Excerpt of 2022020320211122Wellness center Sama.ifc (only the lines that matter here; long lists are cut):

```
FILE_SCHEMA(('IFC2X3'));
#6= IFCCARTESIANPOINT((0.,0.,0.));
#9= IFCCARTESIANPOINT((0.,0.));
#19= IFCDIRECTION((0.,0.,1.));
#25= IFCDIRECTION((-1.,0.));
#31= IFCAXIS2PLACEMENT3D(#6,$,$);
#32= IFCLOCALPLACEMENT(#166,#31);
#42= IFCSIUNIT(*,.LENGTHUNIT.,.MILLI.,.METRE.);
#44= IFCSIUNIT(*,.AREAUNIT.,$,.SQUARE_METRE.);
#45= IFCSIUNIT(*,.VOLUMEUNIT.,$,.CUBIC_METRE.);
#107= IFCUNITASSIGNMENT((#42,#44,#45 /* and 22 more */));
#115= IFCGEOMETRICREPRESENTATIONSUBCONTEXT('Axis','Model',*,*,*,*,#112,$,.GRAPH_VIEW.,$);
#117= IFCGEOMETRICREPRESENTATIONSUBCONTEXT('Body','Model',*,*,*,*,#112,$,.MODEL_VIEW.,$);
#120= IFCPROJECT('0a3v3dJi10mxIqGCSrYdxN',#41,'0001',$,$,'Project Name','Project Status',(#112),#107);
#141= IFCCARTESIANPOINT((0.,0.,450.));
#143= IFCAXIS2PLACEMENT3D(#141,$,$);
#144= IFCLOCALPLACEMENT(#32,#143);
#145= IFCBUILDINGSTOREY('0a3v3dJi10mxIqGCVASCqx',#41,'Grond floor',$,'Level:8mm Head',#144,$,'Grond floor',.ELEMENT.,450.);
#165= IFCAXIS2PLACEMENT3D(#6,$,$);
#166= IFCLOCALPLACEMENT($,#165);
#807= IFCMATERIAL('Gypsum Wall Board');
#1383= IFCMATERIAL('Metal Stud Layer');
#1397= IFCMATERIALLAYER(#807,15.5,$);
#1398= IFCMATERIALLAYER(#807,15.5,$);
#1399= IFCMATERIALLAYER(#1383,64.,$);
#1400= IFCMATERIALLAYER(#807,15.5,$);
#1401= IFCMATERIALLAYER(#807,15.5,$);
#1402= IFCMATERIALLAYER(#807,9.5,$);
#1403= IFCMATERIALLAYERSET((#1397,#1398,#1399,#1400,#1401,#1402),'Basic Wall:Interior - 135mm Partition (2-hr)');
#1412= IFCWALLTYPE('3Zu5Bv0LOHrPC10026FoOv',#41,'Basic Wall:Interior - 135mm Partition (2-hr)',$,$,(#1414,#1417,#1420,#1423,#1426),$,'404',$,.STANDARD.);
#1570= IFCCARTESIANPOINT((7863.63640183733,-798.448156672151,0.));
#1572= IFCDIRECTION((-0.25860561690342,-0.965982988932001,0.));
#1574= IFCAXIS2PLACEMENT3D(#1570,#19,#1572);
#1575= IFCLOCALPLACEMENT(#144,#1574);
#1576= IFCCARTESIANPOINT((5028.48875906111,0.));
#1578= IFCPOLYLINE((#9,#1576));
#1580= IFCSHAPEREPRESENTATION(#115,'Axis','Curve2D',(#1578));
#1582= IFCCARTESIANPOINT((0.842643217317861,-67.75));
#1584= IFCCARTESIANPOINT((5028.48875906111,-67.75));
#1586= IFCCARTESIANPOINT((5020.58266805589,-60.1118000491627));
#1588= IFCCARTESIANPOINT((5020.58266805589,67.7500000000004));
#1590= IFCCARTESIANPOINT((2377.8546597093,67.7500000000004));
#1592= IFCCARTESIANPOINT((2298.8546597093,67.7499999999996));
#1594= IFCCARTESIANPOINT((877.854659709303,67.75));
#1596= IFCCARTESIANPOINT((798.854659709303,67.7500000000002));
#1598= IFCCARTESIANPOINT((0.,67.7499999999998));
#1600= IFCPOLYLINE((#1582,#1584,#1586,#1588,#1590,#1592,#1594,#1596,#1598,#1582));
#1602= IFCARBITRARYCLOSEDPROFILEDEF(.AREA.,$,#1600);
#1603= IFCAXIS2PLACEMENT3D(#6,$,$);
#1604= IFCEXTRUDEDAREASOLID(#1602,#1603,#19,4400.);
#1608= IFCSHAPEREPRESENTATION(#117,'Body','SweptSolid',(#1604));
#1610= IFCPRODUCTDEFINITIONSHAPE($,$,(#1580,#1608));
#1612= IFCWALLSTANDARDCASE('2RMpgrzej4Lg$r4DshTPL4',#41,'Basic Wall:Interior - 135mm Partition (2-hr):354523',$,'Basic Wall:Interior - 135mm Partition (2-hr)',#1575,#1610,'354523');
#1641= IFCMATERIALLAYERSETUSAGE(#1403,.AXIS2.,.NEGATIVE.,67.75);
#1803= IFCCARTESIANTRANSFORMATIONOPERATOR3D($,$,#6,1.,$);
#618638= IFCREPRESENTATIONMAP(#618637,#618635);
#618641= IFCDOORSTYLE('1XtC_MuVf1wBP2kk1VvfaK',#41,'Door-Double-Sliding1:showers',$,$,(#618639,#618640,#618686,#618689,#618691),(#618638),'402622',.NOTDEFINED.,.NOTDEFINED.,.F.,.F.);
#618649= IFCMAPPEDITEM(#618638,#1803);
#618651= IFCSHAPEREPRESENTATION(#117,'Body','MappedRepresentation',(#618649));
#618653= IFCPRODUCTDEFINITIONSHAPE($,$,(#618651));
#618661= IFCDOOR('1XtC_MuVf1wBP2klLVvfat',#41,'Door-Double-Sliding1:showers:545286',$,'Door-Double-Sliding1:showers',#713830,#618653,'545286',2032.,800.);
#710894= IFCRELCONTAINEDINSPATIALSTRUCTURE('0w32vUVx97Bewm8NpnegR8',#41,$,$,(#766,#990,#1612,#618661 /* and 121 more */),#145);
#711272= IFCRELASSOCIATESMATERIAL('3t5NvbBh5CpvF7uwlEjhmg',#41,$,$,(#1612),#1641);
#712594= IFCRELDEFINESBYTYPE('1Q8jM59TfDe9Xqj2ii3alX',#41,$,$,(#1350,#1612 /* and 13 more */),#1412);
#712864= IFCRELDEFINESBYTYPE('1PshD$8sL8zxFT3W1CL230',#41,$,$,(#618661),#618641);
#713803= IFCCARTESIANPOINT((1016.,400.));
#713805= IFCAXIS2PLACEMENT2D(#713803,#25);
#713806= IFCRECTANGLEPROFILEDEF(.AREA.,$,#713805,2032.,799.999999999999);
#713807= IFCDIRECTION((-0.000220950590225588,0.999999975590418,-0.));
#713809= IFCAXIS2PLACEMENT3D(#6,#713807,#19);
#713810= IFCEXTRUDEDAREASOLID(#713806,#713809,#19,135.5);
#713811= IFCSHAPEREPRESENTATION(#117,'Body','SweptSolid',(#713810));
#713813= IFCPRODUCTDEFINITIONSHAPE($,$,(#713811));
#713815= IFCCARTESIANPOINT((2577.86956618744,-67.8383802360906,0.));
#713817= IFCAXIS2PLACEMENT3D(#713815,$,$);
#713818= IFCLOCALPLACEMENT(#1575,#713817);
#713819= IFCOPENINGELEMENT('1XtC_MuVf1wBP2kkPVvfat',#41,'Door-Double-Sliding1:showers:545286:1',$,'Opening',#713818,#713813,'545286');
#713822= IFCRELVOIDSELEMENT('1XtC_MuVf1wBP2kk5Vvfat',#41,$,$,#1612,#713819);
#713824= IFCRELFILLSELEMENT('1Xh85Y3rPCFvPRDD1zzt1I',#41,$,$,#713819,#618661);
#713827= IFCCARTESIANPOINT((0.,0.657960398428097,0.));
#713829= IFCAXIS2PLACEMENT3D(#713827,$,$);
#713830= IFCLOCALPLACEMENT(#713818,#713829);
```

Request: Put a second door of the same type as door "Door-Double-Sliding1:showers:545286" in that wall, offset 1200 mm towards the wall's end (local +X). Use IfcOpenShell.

```python
import ifcopenshell
import ifcopenshell.api.feature
import ifcopenshell.api.geometry
import ifcopenshell.api.root
import ifcopenshell.geom
import ifcopenshell.util.element
import ifcopenshell.util.placement
import ifcopenshell.util.shape
import ifcopenshell.util.unit

model = ifcopenshell.open("2022020320211122Wellness center Sama.ifc")
unit_scale = ifcopenshell.util.unit.calculate_unit_scale(model)
settings = ifcopenshell.geom.settings()


def volume(element):
    """Net volume in cubic metres, openings subtracted."""
    shape = ifcopenshell.geom.create_shape(settings, element)
    return ifcopenshell.util.shape.get_volume(shape.geometry)


def reuse_history(source, copy):
    """copy_class also copies each property set's owner history, people and application; keep the originals."""
    for rel in copy.IsDefinedBy:
        if rel.is_a("IfcRelDefinesByProperties") and (history := rel.RelatingPropertyDefinition.OwnerHistory):
            rel.RelatingPropertyDefinition.OwnerHistory = source.OwnerHistory
            ifcopenshell.util.element.remove_deep2(model, history)


door = model.by_id(618661)
opening = door.FillsVoids[0].RelatingOpeningElement
wall = opening.VoidsElements[0].RelatingBuildingElement
before = volume(wall)
shift = ifcopenshell.util.placement.get_local_placement(wall.ObjectPlacement)[:3, 0] * 1.2 / unit_scale

# copy_class copies the void relationship, type, container and properties, but no geometry.
new_opening = ifcopenshell.api.root.copy_class(model, product=opening)
new_opening.Representation = ifcopenshell.util.element.copy_deep(
    model, opening.Representation, exclude=["IfcGeometricRepresentationContext", "IfcRepresentationMap"]
)
new_opening.Name = "Door-Double-Sliding1:showers"
new_opening.Tag = None
new_door = ifcopenshell.api.root.copy_class(model, product=door)
new_door.Representation = ifcopenshell.util.element.copy_deep(
    model, door.Representation, exclude=["IfcGeometricRepresentationContext", "IfcRepresentationMap"]
)
new_door.Name = "Door-Double-Sliding1:showers"
new_door.Tag = None
reuse_history(door, new_door)
fills = ifcopenshell.api.feature.add_filling(model, opening=new_opening, element=new_door)
fills.OwnerHistory = new_door.OwnerHistory  # required in IFC2X3

for old, new in ((opening, new_opening), (door, new_door)):
    matrix = ifcopenshell.util.placement.get_local_placement(old.ObjectPlacement)
    matrix[:3, 3] += shift
    ifcopenshell.api.geometry.edit_object_placement(model, product=new, matrix=matrix, is_si=False)

after = volume(wall)

print(f"wall volume {before:.3f} -> {after:.3f} m3")

model.write("2022020320211122Wellness center Sama_v2.ifc")
```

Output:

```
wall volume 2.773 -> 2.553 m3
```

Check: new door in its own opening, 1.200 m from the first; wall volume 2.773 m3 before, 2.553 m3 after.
